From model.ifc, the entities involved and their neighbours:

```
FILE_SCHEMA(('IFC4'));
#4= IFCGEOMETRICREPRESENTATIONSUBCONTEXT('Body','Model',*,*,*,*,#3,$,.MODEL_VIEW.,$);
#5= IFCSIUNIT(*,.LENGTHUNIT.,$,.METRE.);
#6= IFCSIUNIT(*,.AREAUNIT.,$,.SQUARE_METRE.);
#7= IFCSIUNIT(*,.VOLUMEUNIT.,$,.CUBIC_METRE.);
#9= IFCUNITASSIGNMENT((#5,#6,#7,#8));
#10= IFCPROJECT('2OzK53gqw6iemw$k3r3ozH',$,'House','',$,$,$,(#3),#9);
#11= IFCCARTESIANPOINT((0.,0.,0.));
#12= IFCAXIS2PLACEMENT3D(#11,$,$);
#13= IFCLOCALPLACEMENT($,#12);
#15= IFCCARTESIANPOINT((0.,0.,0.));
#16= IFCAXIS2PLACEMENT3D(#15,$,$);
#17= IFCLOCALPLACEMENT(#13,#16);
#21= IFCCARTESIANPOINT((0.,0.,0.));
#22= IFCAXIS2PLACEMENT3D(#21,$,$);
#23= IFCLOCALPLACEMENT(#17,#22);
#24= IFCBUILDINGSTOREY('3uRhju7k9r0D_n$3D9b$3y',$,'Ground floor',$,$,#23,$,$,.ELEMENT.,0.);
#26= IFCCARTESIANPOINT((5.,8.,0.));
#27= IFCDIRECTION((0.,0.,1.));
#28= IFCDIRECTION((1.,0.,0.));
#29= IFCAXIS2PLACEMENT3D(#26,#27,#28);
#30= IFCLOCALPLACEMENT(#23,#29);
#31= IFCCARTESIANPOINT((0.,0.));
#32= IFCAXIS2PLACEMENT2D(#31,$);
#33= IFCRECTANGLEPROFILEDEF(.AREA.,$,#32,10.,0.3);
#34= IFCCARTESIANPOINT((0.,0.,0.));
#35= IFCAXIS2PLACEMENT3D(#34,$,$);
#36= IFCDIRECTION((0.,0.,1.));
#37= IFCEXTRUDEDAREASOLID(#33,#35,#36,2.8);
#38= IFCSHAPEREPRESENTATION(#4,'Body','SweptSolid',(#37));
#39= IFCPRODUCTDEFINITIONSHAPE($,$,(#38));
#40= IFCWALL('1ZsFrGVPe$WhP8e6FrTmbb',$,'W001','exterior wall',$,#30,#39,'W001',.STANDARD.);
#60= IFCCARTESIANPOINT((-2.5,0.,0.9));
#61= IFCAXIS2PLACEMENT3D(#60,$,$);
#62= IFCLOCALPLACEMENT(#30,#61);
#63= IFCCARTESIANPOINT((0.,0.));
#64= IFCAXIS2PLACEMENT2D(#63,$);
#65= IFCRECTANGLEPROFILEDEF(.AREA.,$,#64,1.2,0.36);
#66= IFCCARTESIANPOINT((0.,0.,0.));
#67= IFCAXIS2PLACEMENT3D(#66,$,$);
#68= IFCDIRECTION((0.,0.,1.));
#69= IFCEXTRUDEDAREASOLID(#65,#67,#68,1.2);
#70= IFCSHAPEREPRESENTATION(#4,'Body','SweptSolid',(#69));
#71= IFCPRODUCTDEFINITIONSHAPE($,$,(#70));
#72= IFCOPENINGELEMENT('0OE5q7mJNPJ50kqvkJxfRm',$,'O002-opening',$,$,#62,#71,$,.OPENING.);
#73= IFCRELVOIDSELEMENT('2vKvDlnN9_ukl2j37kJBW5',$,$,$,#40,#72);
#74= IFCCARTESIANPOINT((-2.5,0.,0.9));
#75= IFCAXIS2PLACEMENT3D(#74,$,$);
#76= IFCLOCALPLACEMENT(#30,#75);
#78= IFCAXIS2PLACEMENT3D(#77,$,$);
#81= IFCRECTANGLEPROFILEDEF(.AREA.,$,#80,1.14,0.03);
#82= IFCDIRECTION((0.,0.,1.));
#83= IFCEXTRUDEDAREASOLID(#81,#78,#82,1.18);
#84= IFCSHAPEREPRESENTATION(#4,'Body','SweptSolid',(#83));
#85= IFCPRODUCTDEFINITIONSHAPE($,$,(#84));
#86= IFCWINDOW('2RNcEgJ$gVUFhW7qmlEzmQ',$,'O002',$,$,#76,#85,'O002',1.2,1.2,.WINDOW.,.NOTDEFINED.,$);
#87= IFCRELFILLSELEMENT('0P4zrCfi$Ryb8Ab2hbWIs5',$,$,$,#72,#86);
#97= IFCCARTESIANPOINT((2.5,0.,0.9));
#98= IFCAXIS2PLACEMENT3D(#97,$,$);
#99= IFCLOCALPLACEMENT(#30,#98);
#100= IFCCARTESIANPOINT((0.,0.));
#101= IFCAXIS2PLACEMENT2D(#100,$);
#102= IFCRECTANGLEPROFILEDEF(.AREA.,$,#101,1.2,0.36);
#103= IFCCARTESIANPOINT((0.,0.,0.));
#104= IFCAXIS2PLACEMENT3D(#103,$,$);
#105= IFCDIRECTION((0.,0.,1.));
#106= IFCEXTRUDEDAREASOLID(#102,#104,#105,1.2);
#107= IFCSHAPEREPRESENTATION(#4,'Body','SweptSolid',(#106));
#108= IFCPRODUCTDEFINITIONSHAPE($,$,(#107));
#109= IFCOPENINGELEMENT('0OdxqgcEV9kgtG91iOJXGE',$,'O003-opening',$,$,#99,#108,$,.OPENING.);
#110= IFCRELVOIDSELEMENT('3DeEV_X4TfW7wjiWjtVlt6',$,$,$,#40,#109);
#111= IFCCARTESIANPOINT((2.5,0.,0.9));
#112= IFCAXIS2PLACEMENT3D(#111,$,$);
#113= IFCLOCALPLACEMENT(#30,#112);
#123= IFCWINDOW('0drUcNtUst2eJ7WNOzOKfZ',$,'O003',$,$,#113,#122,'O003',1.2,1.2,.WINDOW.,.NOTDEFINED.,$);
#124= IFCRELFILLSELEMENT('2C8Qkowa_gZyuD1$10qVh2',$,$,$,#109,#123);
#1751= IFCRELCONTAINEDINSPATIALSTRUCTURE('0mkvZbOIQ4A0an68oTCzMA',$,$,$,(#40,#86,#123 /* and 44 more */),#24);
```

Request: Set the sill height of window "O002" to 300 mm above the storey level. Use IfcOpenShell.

```python
import numpy as np
import ifcopenshell
import ifcopenshell.api.geometry
import ifcopenshell.geom
import ifcopenshell.util.element
import ifcopenshell.util.placement
import ifcopenshell.util.shape
import ifcopenshell.util.unit

model = ifcopenshell.open("model.ifc")
unit_scale = ifcopenshell.util.unit.calculate_unit_scale(model)

window = model.by_guid("2RNcEgJ$gVUFhW7qmlEzmQ")
opening = window.FillsVoids[0].RelatingOpeningElement
storey = ifcopenshell.util.element.get_container(window, ifc_class="IfcBuildingStorey")
level = ifcopenshell.util.placement.get_local_placement(storey.ObjectPlacement)[2, 3]

# The opening's origin need not be at the sill, so measure its lowest point.
shape = ifcopenshell.geom.create_shape(ifcopenshell.geom.settings(), opening)
bottom = ifcopenshell.util.shape.get_shape_bottom_elevation(shape, shape.geometry) / unit_scale
dz = level + 0.3 / unit_scale - bottom

shift = np.array([0.0, 0.0, dz])
# The window is not placed relative to its opening, so move both.
for product in (opening, window):
    matrix = ifcopenshell.util.placement.get_local_placement(product.ObjectPlacement)
    matrix[:3, 3] += shift
    ifcopenshell.api.geometry.edit_object_placement(model, product=product, matrix=matrix, is_si=False)

print(f"moved by {dz * unit_scale:+.3f} m")

model.write("model_edited.ifc")
```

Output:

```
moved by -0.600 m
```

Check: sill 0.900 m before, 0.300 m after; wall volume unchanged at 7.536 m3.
